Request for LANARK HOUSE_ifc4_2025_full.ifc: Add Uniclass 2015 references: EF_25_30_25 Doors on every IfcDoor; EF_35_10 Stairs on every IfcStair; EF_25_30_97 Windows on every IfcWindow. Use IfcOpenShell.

First a look at what the model holds.

```python
import ifcopenshell

model = ifcopenshell.open("LANARK HOUSE_ifc4_2025_full.ifc")
print(model.schema)
print("classifications:", [c.Name for c in model.by_type("IfcClassification")])
for ifc_class in ("IfcDoor", "IfcRoof", "IfcStair", "IfcWall", "IfcWindow"):
    print(ifc_class, len(model.by_type(ifc_class)))
```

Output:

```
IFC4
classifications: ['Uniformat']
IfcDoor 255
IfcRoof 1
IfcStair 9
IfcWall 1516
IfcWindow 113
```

```python
import ifcopenshell
import ifcopenshell.api.classification

model = ifcopenshell.open("LANARK HOUSE_ifc4_2025_full.ifc")

system = ifcopenshell.api.classification.add_classification(model, classification="Uniclass 2015")

codes = {
    "IfcDoor": ("EF_25_30_25", "Doors"),
    "IfcStair": ("EF_35_10", "Stairs"),
    "IfcWindow": ("EF_25_30_97", "Windows"),
}
for ifc_class, (code, name) in codes.items():
    products = model.by_type(ifc_class)
    ifcopenshell.api.classification.add_reference(
        model, products=products, classification=system, identification=code, name=name
    )
    print(code, len(products))

model.write("LANARK HOUSE_ifc4_2025_full_updated.ifc")
```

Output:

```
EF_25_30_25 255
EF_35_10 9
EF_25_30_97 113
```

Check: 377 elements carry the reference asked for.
